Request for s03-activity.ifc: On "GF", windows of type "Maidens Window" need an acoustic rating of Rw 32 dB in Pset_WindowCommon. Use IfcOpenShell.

First a look at what the model holds.

```python
import ifcopenshell
import ifcopenshell.util.element

model = ifcopenshell.open("s03-activity.ifc")
print(model.schema)
storey = next(s for s in model.by_type("IfcBuildingStorey") if s.Name == "GF")
windows = [e for e in ifcopenshell.util.element.get_decomposition(storey) if e.is_a("IfcWindow")]
seen = {}
for e in windows:
    element_type = ifcopenshell.util.element.get_type(e)
    key = (element_type.Name if element_type != e and element_type else None, ifcopenshell.util.element.get_pset(e, "Pset_WindowCommon", "AcousticRating"))
    seen[key] = seen.get(key, 0) + 1
for (name, value), count in sorted(seen.items(), key=str):
    print(count, "x", name, "|", value)
```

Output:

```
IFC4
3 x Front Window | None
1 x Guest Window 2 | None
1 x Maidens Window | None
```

```python
import ifcopenshell
import ifcopenshell.api.pset
import ifcopenshell.util.element

model = ifcopenshell.open("s03-activity.ifc")

storey = next(s for s in model.by_type("IfcBuildingStorey") if s.Name == "GF")
windows = [e for e in ifcopenshell.util.element.get_decomposition(storey) if e.is_a("IfcWindow")]

count = 0
for e in windows:
    element_type = ifcopenshell.util.element.get_type(e)
    if element_type in (None, e) or element_type.Name != "Maidens Window":
        continue
    # add_pset returns the element's existing set when there is one.
    pset = ifcopenshell.api.pset.add_pset(model, product=e, name="Pset_WindowCommon")
    ifcopenshell.api.pset.edit_pset(model, pset=pset, properties={"AcousticRating": "Rw 32 dB"})
    count += 1

print(count, "windows updated")

model.write("s03-activity_edited.ifc")
```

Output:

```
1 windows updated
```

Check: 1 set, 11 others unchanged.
